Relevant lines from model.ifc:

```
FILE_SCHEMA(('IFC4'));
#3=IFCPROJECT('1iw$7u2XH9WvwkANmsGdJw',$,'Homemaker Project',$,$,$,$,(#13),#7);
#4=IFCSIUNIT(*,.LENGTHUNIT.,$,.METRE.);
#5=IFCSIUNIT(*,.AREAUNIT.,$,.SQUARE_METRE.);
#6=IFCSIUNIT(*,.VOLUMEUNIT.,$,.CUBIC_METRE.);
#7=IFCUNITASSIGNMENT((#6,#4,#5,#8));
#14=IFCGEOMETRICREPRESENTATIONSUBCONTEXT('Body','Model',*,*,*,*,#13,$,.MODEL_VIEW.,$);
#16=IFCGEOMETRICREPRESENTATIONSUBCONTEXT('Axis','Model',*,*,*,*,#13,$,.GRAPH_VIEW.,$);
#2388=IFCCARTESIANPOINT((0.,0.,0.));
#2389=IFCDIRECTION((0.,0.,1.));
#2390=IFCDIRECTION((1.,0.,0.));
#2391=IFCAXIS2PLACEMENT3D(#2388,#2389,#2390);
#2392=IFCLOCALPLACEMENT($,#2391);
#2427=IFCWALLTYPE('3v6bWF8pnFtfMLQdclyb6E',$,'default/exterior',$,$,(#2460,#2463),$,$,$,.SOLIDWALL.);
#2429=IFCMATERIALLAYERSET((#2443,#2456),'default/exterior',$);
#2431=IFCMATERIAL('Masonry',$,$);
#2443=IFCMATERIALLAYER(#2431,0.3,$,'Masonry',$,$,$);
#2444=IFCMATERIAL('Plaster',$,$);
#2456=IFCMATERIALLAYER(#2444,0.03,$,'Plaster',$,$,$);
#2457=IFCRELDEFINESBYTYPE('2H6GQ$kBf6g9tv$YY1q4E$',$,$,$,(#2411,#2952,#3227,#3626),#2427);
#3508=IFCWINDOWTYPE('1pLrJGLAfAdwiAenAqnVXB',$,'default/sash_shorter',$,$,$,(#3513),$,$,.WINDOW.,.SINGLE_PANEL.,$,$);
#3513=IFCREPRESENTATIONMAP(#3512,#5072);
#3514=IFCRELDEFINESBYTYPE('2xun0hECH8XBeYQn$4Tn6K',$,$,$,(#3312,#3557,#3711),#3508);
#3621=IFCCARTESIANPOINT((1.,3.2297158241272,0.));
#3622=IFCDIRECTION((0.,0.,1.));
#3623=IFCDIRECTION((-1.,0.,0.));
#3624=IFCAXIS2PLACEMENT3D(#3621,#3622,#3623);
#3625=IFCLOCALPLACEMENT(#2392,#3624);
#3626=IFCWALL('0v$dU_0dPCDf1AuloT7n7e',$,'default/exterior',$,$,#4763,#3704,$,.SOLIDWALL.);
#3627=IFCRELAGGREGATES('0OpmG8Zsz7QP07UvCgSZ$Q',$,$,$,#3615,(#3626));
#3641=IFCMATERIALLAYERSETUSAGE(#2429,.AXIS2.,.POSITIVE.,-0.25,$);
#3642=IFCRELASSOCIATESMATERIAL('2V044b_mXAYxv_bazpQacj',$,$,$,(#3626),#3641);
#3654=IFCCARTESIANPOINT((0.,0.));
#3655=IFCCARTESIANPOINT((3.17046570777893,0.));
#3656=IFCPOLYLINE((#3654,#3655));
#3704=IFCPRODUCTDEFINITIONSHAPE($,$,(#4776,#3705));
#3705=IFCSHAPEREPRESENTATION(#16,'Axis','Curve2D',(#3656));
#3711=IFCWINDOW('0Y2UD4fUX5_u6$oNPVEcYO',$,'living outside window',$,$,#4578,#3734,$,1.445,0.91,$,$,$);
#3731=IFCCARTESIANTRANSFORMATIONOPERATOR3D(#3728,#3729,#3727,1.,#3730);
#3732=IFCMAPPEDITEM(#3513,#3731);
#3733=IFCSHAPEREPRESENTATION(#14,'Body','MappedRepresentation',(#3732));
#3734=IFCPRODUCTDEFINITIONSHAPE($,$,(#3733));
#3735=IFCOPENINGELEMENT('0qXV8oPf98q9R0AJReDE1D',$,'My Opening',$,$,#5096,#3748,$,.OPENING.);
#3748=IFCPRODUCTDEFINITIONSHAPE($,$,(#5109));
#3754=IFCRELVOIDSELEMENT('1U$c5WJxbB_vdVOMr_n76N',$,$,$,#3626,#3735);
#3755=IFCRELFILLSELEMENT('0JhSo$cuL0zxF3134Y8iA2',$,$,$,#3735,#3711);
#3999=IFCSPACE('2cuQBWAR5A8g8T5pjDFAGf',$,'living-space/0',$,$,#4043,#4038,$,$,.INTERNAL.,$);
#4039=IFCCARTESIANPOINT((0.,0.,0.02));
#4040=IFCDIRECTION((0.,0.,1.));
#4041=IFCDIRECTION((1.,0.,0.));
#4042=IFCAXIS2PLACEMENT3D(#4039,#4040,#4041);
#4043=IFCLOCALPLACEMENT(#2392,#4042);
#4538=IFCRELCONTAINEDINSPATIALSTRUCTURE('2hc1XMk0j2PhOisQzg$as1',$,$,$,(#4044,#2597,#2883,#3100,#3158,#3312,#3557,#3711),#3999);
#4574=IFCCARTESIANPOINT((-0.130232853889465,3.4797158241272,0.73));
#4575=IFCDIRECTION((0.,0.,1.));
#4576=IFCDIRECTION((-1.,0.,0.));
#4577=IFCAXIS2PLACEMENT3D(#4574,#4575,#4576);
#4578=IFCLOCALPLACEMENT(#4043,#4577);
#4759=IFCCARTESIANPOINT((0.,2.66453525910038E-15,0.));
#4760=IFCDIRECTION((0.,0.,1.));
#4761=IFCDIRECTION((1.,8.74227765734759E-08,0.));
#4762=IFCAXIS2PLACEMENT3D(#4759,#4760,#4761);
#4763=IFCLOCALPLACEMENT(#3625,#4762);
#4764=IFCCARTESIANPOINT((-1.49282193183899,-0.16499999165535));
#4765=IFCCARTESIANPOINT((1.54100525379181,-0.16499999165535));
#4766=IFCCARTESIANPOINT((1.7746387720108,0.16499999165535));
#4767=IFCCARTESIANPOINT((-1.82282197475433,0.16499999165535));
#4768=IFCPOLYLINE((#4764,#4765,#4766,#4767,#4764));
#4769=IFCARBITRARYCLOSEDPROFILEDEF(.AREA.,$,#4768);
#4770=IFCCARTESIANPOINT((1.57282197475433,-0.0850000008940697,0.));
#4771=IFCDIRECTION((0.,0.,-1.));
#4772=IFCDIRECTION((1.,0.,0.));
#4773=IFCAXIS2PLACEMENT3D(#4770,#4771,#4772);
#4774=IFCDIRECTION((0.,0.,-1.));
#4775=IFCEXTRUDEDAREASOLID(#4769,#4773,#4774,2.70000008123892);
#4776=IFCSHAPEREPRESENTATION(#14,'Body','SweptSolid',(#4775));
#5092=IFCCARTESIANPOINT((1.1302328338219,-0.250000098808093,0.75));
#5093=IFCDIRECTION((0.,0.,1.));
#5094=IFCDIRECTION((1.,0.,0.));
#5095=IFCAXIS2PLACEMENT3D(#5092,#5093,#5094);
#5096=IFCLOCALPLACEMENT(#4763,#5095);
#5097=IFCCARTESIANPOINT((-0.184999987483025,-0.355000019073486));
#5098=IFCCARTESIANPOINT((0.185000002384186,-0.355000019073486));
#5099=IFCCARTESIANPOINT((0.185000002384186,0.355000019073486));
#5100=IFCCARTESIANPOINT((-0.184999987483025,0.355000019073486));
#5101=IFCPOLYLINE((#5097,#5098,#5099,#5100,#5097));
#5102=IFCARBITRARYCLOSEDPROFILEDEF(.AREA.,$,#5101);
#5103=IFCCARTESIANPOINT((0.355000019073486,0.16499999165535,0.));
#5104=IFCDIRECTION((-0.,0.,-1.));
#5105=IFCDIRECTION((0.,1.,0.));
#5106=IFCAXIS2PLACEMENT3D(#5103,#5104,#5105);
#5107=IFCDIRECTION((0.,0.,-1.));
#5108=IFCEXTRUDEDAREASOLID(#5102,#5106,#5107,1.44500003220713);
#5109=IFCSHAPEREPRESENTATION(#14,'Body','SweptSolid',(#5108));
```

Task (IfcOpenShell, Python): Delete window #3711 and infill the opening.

```python
import ifcopenshell
import ifcopenshell.api.feature
import ifcopenshell.api.root
import ifcopenshell.geom
import ifcopenshell.util.shape

model = ifcopenshell.open("model.ifc")
settings = ifcopenshell.geom.settings()


def volume(element):
    """Net volume in cubic metres, openings subtracted."""
    shape = ifcopenshell.geom.create_shape(settings, element)
    return ifcopenshell.util.shape.get_volume(shape.geometry)


window = model.by_guid("0Y2UD4fUX5_u6$oNPVEcYO")
opening = window.FillsVoids[0].RelatingOpeningElement
wall = opening.VoidsElements[0].RelatingBuildingElement
before = volume(wall)

ifcopenshell.api.root.remove_product(model, product=window)
ifcopenshell.api.feature.remove_feature(model, feature=opening)

after = volume(wall)

print(f"wall volume {before:.3f} -> {after:.3f} m3")

model.write("model_edited.ifc")
```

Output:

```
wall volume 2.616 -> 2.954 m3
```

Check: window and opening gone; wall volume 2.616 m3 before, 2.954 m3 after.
